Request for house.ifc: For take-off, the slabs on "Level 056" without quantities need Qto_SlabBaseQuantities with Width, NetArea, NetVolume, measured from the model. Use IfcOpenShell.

First a look at what the model holds.

```python
import ifcopenshell
import ifcopenshell.util.element
import ifcopenshell.util.unit

model = ifcopenshell.open("house.ifc")
print(model.schema)
for unit_type in ("LENGTHUNIT", "AREAUNIT", "VOLUMEUNIT"):
    print(unit_type, ifcopenshell.util.unit.calculate_unit_scale(model, unit_type))
storey = next(s for s in model.by_type("IfcBuildingStorey") if s.Name == "Level 056")
slabs = [e for e in ifcopenshell.util.element.get_decomposition(storey) if e.is_a("IfcSlab")]
for e in sorted(slabs, key=lambda e: e.id()):
    print(e.id(), e.is_a(), e.Name, list(ifcopenshell.util.element.get_psets(e, qtos_only=True)), sep=" | ")
```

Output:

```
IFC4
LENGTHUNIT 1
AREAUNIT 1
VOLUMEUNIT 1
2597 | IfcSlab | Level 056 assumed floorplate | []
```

```python
import ifcopenshell
import ifcopenshell.api.pset
import ifcopenshell.geom
import ifcopenshell.util.element
import ifcopenshell.util.shape
import ifcopenshell.util.unit

model = ifcopenshell.open("house.ifc")
unit_scale = ifcopenshell.util.unit.calculate_unit_scale(model)
area_scale = ifcopenshell.util.unit.calculate_unit_scale(model, "AREAUNIT")
volume_scale = ifcopenshell.util.unit.calculate_unit_scale(model, "VOLUMEUNIT")
settings = ifcopenshell.geom.settings()

storey = next(s for s in model.by_type("IfcBuildingStorey") if s.Name == "Level 056")
slabs = [e for e in ifcopenshell.util.element.get_decomposition(storey) if e.is_a("IfcSlab")]

for e in sorted(slabs, key=lambda e: e.id()):
    if ifcopenshell.util.element.get_psets(e, qtos_only=True, should_inherit=False):
        continue
    # Geometry comes back in metres, in the element's own axes.
    shape = ifcopenshell.geom.create_shape(settings, e)
    values = {
        "Width": ifcopenshell.util.shape.get_z(shape.geometry) / unit_scale,
        "NetArea": ifcopenshell.util.shape.get_footprint_area(shape.geometry) / area_scale,
        "NetVolume": ifcopenshell.util.shape.get_volume(shape.geometry) / volume_scale,
    }
    qto = ifcopenshell.api.pset.add_qto(model, product=e, name="Qto_SlabBaseQuantities")
    ifcopenshell.api.pset.edit_qto(model, qto=qto, properties=values)
    print(e.id(), {k: round(v, 3) for k, v in values.items()})

model.write("house_edited.ifc")
```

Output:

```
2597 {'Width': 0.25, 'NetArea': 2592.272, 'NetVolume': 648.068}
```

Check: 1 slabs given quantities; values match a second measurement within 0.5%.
